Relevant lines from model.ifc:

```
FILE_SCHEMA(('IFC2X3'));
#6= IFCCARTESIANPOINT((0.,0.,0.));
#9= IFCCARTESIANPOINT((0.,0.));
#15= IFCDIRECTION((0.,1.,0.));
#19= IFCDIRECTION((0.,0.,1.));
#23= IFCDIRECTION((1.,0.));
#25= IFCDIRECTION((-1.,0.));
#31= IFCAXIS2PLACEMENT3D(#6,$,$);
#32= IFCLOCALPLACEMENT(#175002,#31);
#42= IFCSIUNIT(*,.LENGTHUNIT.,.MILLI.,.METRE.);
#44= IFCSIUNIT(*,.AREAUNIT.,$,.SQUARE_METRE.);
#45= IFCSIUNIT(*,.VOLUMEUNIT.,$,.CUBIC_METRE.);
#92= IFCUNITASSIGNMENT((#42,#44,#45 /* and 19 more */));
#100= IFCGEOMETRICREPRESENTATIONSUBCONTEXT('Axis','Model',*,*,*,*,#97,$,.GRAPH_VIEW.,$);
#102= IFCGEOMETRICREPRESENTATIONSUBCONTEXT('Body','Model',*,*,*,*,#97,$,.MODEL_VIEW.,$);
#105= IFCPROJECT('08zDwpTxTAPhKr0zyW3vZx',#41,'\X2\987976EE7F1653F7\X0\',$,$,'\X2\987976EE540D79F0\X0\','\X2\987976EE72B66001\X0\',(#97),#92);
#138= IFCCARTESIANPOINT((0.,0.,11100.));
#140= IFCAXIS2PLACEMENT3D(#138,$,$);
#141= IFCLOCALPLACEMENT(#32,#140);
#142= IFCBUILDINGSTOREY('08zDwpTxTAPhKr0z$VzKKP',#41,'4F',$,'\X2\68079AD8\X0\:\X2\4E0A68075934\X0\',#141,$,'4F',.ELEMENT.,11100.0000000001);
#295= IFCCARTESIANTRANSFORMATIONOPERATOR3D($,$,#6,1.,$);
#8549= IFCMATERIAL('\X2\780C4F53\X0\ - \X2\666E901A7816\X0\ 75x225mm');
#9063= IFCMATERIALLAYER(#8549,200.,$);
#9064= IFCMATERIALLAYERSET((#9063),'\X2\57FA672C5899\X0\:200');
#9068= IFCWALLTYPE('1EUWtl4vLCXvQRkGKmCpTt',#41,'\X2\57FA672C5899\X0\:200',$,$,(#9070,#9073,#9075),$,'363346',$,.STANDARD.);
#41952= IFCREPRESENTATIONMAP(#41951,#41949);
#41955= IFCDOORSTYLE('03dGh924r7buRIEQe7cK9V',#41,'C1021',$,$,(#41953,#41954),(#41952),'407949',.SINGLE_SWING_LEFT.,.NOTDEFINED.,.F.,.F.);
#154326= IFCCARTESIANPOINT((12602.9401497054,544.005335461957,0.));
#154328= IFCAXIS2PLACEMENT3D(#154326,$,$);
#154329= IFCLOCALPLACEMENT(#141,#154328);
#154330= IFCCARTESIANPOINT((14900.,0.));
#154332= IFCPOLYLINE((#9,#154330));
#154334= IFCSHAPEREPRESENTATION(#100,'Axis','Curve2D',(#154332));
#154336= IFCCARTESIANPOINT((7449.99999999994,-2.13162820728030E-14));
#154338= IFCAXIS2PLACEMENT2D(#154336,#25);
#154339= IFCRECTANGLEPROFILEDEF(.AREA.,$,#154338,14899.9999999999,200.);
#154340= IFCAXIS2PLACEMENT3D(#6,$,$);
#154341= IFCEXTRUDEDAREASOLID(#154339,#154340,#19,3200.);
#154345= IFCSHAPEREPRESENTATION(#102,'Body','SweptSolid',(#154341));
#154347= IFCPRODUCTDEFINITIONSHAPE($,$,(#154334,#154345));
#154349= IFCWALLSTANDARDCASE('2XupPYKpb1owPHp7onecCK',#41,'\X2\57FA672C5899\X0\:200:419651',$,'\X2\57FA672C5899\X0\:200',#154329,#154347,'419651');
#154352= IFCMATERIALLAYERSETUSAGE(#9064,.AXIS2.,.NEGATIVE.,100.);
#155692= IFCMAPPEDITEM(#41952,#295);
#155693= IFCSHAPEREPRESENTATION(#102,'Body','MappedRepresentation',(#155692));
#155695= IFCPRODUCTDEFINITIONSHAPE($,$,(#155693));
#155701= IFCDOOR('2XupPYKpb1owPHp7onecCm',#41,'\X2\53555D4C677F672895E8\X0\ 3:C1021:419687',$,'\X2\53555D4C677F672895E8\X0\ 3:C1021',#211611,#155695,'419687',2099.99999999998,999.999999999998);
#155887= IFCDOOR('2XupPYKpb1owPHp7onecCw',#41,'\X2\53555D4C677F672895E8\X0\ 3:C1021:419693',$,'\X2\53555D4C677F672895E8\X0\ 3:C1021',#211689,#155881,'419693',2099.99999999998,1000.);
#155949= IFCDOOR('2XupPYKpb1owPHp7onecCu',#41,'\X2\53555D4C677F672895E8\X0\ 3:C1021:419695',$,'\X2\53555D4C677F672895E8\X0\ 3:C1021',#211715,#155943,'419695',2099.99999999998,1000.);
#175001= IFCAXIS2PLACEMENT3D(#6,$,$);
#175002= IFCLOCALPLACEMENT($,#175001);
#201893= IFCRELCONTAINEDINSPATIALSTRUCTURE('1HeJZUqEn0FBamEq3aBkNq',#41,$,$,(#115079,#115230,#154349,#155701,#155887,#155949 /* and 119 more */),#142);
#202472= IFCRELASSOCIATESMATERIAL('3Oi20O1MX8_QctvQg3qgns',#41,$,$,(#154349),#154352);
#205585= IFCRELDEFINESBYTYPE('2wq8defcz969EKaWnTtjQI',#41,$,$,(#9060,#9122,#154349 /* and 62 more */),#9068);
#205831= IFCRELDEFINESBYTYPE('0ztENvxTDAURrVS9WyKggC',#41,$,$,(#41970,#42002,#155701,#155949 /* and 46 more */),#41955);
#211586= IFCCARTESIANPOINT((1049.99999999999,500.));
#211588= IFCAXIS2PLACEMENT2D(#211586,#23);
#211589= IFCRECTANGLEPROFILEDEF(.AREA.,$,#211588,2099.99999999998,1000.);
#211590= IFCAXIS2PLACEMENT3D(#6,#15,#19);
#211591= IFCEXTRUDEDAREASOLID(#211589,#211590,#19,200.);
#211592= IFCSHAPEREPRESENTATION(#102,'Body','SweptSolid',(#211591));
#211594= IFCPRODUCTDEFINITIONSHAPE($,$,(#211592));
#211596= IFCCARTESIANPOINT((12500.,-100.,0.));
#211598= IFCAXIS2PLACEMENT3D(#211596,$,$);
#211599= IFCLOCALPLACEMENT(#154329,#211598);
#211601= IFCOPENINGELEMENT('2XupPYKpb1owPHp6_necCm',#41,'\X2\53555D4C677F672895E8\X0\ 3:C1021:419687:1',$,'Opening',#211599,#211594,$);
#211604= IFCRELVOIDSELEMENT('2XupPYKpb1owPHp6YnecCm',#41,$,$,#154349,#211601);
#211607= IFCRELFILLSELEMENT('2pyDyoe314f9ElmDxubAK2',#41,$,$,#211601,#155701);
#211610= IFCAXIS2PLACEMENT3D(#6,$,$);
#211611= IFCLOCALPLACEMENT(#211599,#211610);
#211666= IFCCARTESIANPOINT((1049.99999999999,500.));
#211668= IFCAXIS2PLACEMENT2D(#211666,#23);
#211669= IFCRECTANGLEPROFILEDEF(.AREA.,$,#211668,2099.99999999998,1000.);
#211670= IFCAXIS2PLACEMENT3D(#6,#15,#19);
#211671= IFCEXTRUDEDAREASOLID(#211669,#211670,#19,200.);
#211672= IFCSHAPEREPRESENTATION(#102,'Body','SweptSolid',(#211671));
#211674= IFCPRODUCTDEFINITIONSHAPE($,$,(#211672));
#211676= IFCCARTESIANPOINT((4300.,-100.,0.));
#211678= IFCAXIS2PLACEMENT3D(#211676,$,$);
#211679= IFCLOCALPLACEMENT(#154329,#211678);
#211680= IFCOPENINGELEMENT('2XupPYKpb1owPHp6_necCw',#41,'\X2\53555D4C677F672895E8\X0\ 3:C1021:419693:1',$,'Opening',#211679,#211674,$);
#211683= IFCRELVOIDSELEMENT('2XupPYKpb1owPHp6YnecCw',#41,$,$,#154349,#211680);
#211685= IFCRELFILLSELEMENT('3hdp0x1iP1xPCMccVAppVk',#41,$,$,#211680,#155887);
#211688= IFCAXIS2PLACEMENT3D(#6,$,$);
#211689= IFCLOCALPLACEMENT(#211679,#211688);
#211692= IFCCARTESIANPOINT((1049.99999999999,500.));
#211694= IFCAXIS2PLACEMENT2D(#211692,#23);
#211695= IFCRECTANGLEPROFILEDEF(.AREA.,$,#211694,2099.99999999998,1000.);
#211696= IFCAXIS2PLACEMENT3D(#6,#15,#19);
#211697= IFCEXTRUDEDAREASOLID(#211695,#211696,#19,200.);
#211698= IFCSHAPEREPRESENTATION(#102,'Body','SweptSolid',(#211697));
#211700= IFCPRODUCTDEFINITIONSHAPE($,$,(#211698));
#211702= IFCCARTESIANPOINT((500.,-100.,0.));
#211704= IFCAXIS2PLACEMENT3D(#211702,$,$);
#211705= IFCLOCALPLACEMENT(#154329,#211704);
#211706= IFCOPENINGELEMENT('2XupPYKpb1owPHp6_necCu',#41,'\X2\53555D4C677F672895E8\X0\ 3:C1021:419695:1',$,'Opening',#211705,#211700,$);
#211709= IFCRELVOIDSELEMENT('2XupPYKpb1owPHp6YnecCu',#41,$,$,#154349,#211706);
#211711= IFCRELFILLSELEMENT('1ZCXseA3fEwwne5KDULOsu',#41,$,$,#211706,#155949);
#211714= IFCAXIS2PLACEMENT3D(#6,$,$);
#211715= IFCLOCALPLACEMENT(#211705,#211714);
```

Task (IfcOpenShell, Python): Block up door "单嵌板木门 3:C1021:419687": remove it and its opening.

```python
import ifcopenshell
import ifcopenshell.api.feature
import ifcopenshell.api.root
import ifcopenshell.geom
import ifcopenshell.util.shape

model = ifcopenshell.open("model.ifc")
settings = ifcopenshell.geom.settings()


def volume(element):
    """Net volume in cubic metres, openings subtracted."""
    shape = ifcopenshell.geom.create_shape(settings, element)
    return ifcopenshell.util.shape.get_volume(shape.geometry)


door = model.by_guid("2XupPYKpb1owPHp7onecCm")
opening = door.FillsVoids[0].RelatingOpeningElement
wall = opening.VoidsElements[0].RelatingBuildingElement
before = volume(wall)

ifcopenshell.api.root.remove_product(model, product=door)
ifcopenshell.api.feature.remove_feature(model, feature=opening)

after = volume(wall)

print(f"wall volume {before:.3f} -> {after:.3f} m3")

model.write("model_updated.ifc")
```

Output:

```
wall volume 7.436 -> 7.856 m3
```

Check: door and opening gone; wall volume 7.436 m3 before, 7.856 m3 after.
